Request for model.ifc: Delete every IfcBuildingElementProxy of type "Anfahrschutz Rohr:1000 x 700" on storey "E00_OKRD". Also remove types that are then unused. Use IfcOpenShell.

First a look at what the model holds.

```python
import ifcopenshell
import ifcopenshell.util.element

model = ifcopenshell.open("model.ifc")
print(model.schema)
storey = next(s for s in model.by_type("IfcBuildingStorey") if s.Name == "E00_OKRD")
proxies = [e for e in ifcopenshell.util.element.get_decomposition(storey) if e.is_a("IfcBuildingElementProxy")]
seen = {}
for e in proxies:
    element_type = ifcopenshell.util.element.get_type(e)
    name = element_type.Name if element_type not in (None, e) else None
    seen[name] = seen.get(name, 0) + 1
for name, count in sorted(seen.items(), key=str):
    print(count, "x", name)
```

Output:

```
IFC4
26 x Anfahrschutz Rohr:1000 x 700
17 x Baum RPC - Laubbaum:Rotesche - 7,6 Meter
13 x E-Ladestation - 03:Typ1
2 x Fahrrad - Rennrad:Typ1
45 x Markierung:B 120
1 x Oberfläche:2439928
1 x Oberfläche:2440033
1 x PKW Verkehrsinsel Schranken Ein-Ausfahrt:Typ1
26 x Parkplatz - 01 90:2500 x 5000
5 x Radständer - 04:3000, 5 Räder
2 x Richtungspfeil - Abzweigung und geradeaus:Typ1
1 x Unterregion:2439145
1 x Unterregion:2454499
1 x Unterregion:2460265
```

```python
import ifcopenshell
import ifcopenshell.api.root
import ifcopenshell.util.element

model = ifcopenshell.open("model.ifc")

storey = next(s for s in model.by_type("IfcBuildingStorey") if s.Name == "E00_OKRD")
proxies = [e for e in ifcopenshell.util.element.get_decomposition(storey) if e.is_a("IfcBuildingElementProxy")]
targets = [e for e in proxies if (t := ifcopenshell.util.element.get_type(e)) not in (None, e) and t.Name == "Anfahrschutz Rohr:1000 x 700"]
types = {ifcopenshell.util.element.get_type(e) for e in targets} - {None, *targets}

for e in targets:
    ifcopenshell.api.root.remove_product(model, product=e)
print(len(targets), "removed")

unused = [t for t in types if not ifcopenshell.util.element.get_types(t)]
for t in unused:
    ifcopenshell.api.root.remove_product(model, product=t)
print(len(unused), "unused types removed")

model.write("model_rev.ifc")
```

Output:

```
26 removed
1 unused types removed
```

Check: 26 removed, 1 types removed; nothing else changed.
